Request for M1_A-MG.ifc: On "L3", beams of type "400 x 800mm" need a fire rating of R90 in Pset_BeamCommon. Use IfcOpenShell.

First a look at what the model holds.

```python
import ifcopenshell
import ifcopenshell.util.element

model = ifcopenshell.open("M1_A-MG.ifc")
print(model.schema)
storey = next(s for s in model.by_type("IfcBuildingStorey") if s.Name == "L3")
beams = [e for e in ifcopenshell.util.element.get_decomposition(storey) if e.is_a("IfcBeam")]
seen = {}
for e in beams:
    element_type = ifcopenshell.util.element.get_type(e)
    key = (element_type.Name if element_type != e and element_type else None, ifcopenshell.util.element.get_pset(e, "Pset_BeamCommon", "FireRating"))
    seen[key] = seen.get(key, 0) + 1
for (name, value), count in sorted(seen.items(), key=str):
    print(count, "x", name, "|", value)
```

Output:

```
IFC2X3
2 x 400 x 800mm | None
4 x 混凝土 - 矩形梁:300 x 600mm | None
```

```python
import ifcopenshell
import ifcopenshell.api.pset
import ifcopenshell.util.element

model = ifcopenshell.open("M1_A-MG.ifc")

storey = next(s for s in model.by_type("IfcBuildingStorey") if s.Name == "L3")
beams = [e for e in ifcopenshell.util.element.get_decomposition(storey) if e.is_a("IfcBeam")]

count = 0
for e in beams:
    element_type = ifcopenshell.util.element.get_type(e)
    if element_type in (None, e) or element_type.Name != "400 x 800mm":
        continue
    # add_pset returns the element's existing set when there is one.
    pset = ifcopenshell.api.pset.add_pset(model, product=e, name="Pset_BeamCommon")
    ifcopenshell.api.pset.edit_pset(model, pset=pset, properties={"FireRating": "R90"})
    count += 1

print(count, "beams updated")

model.write("M1_A-MG_edited.ifc")
```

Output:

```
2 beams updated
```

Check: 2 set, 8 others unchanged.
